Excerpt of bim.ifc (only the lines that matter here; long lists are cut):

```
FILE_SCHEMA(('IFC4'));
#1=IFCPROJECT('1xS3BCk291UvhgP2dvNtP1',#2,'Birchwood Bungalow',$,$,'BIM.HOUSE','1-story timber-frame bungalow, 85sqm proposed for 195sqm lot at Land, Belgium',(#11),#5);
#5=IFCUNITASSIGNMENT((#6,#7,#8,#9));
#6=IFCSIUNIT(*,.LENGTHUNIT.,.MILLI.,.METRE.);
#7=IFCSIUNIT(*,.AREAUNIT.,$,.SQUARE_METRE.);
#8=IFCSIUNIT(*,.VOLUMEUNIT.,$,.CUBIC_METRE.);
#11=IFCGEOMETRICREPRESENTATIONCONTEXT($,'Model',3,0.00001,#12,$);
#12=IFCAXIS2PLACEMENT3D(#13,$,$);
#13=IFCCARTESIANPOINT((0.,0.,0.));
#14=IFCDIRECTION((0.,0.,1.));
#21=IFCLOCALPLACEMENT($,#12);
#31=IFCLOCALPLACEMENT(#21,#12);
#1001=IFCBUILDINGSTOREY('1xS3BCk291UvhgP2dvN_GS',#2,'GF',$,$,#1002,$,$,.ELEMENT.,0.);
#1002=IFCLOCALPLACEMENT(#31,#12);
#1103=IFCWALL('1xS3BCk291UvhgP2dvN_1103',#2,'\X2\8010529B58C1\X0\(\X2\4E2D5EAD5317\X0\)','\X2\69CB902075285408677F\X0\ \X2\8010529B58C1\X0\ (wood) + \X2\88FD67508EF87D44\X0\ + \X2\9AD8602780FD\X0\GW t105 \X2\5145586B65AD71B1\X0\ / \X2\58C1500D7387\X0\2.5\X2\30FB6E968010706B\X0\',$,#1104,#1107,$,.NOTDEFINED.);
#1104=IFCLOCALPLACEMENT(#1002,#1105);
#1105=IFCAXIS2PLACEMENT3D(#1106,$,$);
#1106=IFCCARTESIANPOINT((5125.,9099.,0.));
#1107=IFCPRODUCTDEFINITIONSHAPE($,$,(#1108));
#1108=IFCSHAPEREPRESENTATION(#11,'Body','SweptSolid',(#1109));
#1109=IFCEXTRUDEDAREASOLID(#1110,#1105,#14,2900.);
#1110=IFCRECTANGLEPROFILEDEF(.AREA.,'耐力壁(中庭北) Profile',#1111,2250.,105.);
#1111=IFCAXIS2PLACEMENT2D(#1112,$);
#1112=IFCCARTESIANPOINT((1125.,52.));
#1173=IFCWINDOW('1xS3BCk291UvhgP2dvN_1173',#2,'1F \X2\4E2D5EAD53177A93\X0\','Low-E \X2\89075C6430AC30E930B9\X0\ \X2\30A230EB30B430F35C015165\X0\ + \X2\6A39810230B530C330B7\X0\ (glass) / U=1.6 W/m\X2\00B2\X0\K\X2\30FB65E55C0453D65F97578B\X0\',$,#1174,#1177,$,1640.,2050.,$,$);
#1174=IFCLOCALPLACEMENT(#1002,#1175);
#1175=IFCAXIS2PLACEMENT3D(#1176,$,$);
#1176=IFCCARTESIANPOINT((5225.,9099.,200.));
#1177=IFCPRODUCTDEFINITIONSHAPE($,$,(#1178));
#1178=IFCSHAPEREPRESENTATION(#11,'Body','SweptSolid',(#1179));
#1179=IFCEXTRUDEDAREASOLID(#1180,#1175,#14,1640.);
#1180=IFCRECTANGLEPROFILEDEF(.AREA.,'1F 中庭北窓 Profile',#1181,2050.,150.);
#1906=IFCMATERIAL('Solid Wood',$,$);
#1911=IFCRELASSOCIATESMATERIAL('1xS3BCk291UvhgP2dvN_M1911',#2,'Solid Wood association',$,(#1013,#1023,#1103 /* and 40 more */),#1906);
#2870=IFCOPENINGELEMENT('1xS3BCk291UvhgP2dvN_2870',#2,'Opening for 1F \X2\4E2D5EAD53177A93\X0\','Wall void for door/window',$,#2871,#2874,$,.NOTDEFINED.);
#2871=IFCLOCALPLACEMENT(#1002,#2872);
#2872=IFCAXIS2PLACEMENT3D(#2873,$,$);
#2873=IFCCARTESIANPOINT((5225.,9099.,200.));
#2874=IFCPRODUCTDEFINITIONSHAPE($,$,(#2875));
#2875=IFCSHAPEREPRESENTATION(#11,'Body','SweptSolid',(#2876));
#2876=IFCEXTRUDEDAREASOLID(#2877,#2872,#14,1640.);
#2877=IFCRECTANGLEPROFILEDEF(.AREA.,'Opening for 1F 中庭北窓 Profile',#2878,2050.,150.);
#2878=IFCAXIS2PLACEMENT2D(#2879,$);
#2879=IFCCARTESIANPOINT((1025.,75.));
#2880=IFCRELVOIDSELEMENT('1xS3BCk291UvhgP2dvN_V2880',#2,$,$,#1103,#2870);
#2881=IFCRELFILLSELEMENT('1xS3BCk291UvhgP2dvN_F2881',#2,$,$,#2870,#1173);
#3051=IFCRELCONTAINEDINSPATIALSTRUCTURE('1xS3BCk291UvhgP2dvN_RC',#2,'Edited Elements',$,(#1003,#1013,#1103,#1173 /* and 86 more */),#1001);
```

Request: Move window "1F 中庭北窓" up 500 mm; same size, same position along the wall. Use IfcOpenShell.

```python
import numpy as np
import ifcopenshell
import ifcopenshell.api.geometry
import ifcopenshell.util.placement
import ifcopenshell.util.unit

model = ifcopenshell.open("bim.ifc")
unit_scale = ifcopenshell.util.unit.calculate_unit_scale(model)

window = model.by_guid("1xS3BCk291UvhgP2dvN_1173")
opening = window.FillsVoids[0].RelatingOpeningElement
dz = 500.0

shift = np.array([0.0, 0.0, dz])
# The window is not placed relative to its opening, so move both.
for product in (opening, window):
    matrix = ifcopenshell.util.placement.get_local_placement(product.ObjectPlacement)
    matrix[:3, 3] += shift
    ifcopenshell.api.geometry.edit_object_placement(model, product=product, matrix=matrix, is_si=False)

print(f"moved by {dz * unit_scale:+.3f} m")

model.write("bim_updated.ifc")
```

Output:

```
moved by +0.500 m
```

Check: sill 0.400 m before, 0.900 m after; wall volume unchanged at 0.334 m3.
